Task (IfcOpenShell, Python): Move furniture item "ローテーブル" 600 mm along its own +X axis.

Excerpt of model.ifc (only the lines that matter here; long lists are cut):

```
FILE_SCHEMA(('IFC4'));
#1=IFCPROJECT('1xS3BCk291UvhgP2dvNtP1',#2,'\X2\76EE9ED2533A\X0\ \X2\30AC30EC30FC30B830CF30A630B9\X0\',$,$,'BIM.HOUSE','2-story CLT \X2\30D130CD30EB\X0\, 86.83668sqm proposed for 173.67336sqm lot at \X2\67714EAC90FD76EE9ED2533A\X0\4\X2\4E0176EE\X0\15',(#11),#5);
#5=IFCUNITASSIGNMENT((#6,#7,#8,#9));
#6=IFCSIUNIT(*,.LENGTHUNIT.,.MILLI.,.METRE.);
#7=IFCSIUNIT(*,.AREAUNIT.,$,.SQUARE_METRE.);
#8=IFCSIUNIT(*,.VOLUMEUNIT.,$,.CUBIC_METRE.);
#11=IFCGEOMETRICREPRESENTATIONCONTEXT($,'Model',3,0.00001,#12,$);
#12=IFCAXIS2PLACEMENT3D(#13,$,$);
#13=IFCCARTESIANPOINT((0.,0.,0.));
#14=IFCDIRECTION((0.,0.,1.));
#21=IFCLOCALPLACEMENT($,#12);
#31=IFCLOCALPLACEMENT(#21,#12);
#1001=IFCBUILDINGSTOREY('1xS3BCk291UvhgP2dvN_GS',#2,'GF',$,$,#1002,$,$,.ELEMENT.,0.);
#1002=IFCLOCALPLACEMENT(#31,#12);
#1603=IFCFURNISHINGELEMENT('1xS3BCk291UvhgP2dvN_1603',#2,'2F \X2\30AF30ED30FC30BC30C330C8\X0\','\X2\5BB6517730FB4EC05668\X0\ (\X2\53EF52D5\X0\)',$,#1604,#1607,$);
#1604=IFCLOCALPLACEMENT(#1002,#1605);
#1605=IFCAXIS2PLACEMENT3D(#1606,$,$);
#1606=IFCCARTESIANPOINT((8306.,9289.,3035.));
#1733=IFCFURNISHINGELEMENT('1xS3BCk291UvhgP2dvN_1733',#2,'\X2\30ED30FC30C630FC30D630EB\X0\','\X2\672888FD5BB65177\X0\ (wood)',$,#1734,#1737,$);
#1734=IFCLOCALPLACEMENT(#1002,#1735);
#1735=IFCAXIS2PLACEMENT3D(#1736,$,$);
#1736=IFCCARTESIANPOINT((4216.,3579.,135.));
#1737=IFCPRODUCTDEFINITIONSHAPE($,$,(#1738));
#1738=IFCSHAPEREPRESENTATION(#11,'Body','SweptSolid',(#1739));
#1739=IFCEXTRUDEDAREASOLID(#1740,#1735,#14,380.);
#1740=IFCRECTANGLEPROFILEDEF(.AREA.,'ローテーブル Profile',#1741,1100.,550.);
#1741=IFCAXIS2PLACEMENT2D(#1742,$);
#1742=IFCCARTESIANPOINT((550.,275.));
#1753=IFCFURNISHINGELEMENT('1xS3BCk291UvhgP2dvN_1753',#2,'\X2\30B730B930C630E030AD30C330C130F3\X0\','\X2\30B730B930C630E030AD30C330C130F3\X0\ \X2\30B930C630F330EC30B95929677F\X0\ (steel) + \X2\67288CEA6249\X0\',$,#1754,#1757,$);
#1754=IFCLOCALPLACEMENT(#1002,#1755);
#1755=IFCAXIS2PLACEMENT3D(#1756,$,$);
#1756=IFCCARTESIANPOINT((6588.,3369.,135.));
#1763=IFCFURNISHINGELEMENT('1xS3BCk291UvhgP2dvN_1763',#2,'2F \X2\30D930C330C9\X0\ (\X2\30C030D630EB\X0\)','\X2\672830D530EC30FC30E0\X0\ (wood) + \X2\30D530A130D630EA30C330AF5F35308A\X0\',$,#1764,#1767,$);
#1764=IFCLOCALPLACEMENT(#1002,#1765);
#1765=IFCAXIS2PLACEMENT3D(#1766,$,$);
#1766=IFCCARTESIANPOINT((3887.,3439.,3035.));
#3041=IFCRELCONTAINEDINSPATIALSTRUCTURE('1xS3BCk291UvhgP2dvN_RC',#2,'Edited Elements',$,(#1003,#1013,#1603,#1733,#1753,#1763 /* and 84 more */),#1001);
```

```python
import ifcopenshell
import ifcopenshell.api.geometry
import ifcopenshell.util.placement

model = ifcopenshell.open("model.ifc")

item = model.by_guid("1xS3BCk291UvhgP2dvN_1733")
matrix = ifcopenshell.util.placement.get_local_placement(item.ObjectPlacement)
matrix[:3, 3] += matrix[:3, 0] * 600.0
ifcopenshell.api.geometry.edit_object_placement(model, product=item, matrix=matrix, is_si=False)

print(ifcopenshell.util.placement.get_local_placement(item.ObjectPlacement).round(3) + 0.0)

model.write("model-out.ifc")
```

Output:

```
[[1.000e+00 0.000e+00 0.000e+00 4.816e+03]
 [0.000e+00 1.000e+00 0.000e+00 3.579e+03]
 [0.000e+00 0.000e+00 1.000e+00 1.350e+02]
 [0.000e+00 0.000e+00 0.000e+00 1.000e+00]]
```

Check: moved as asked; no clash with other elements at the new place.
